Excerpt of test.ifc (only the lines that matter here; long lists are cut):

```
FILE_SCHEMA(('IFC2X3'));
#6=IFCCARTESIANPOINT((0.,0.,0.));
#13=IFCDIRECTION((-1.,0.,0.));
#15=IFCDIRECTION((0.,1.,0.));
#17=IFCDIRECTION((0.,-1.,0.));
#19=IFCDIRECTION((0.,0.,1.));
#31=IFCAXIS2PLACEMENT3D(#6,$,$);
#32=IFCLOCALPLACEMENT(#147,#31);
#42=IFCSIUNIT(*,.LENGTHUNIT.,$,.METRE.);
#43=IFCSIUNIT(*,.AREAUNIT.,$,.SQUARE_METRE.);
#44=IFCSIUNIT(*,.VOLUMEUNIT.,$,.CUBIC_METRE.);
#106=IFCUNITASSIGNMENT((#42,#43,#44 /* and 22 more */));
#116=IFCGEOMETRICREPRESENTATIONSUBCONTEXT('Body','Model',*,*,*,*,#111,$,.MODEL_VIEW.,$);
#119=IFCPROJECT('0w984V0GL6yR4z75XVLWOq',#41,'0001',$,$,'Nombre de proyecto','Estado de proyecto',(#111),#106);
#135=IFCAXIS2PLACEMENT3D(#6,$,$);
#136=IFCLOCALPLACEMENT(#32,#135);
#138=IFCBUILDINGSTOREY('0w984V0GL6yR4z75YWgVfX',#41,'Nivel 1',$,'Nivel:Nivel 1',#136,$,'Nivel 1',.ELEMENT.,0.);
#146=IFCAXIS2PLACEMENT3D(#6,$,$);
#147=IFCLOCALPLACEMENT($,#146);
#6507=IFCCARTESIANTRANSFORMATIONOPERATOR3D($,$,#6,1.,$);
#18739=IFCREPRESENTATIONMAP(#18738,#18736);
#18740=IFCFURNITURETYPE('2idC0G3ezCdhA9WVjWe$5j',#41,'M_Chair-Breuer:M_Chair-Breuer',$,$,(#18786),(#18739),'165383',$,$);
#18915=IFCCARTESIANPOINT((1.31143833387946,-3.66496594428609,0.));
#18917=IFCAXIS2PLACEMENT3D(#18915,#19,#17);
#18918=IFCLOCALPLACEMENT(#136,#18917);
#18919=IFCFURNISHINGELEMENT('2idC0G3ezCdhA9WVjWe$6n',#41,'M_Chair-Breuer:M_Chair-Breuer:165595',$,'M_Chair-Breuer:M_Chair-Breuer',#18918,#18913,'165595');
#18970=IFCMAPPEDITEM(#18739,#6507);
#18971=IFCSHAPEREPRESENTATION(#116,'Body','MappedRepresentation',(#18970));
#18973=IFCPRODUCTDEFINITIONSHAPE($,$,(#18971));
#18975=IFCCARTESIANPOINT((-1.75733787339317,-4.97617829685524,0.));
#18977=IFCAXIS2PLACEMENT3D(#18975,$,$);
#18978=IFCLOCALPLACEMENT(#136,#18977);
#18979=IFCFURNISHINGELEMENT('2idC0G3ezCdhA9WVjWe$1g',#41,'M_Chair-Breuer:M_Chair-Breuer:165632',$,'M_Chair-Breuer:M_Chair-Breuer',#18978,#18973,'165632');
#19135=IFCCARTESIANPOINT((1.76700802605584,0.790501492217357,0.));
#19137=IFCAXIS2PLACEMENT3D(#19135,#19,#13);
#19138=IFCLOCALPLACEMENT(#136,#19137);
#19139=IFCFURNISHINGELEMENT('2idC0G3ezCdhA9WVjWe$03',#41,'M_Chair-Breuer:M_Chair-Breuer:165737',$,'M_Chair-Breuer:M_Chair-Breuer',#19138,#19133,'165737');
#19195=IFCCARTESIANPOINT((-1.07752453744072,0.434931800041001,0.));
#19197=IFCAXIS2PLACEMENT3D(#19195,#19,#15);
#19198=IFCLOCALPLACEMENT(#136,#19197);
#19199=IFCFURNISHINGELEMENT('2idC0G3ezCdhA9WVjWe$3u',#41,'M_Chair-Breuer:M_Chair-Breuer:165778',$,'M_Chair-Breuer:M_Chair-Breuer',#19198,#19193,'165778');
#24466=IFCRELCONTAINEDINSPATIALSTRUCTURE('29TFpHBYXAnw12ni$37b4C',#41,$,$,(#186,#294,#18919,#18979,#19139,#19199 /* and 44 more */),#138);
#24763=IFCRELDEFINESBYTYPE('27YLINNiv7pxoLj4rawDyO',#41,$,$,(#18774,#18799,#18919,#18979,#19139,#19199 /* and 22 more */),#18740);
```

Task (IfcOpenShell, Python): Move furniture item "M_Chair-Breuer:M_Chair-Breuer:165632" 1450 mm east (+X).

```python
import ifcopenshell
import ifcopenshell.api.geometry
import ifcopenshell.util.placement

model = ifcopenshell.open("test.ifc")

item = model.by_id(18979)
matrix = ifcopenshell.util.placement.get_local_placement(item.ObjectPlacement)
matrix[0, 3] += 1.45
ifcopenshell.api.geometry.edit_object_placement(model, product=item, matrix=matrix, is_si=False)

print(ifcopenshell.util.placement.get_local_placement(item.ObjectPlacement).round(3) + 0.0)

model.write("test_v2.ifc")
```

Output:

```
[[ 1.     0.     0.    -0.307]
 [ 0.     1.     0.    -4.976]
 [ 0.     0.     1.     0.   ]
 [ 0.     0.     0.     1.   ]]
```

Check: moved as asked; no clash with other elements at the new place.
